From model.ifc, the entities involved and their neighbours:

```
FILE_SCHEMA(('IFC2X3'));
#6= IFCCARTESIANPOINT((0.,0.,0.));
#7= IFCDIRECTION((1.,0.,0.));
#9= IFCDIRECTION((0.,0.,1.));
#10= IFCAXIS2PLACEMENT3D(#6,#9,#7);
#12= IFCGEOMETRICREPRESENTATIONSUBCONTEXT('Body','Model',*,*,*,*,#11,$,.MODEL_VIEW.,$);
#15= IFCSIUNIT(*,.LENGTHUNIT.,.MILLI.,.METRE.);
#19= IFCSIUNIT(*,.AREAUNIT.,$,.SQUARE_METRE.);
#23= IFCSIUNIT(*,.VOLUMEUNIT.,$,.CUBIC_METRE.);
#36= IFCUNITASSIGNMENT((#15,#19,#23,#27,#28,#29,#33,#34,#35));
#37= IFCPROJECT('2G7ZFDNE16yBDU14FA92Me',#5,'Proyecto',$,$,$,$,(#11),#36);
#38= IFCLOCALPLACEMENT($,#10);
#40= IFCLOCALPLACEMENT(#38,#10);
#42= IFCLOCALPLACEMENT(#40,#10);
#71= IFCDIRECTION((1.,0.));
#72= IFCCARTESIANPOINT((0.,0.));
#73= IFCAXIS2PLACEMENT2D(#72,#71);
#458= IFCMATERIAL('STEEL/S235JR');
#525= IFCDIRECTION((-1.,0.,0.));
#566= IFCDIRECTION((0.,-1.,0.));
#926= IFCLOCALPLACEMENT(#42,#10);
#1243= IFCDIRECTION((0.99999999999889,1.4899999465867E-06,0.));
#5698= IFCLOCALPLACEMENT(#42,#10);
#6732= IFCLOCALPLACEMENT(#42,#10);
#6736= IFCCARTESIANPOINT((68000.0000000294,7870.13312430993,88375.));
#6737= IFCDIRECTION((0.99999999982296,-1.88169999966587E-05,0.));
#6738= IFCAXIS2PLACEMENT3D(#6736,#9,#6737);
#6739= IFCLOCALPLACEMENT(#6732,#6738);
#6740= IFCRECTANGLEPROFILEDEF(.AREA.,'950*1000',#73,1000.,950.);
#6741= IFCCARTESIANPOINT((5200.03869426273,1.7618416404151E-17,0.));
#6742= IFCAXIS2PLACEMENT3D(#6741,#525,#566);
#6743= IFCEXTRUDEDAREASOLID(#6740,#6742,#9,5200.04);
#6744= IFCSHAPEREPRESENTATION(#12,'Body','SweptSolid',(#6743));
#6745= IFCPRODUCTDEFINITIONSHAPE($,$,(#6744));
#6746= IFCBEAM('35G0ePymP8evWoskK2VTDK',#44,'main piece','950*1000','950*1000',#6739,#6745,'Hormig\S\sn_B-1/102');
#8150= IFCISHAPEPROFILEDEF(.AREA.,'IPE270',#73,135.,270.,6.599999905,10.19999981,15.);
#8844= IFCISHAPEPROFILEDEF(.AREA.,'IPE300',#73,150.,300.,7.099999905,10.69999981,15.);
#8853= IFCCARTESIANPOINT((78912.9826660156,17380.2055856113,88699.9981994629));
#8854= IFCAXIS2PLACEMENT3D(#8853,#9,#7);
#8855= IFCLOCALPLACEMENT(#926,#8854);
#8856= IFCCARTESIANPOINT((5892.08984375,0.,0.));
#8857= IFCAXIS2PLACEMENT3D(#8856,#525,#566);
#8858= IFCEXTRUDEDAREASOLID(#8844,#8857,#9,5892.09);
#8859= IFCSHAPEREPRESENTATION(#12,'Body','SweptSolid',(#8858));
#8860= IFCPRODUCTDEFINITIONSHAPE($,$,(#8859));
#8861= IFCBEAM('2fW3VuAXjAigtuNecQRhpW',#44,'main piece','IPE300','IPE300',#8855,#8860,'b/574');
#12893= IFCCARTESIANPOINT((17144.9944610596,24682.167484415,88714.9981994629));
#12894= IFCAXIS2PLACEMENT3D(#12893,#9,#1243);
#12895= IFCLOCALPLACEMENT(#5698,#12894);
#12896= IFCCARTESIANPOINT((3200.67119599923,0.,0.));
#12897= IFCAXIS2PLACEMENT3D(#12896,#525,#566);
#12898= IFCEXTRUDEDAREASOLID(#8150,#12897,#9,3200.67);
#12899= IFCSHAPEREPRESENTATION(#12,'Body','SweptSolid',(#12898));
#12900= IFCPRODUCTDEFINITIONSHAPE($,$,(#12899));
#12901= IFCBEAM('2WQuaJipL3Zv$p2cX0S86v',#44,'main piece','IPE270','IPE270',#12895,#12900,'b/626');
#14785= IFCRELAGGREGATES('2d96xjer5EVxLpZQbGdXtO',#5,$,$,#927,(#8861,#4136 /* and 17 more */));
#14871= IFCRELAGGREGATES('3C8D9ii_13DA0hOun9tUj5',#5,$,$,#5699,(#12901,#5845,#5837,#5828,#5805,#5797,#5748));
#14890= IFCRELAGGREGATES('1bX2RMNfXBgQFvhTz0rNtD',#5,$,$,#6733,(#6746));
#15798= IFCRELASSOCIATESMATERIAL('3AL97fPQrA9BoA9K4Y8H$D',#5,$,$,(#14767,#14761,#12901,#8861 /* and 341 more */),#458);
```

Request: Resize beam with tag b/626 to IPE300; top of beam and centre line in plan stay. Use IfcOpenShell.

```python
import ifcopenshell
import ifcopenshell.util.element
import ifcopenshell.util.representation

model = ifcopenshell.open("model.ifc")

member = model.by_id(12901)
source = next(p for p in model.by_type("IfcIShapeProfileDef") if p.ProfileName == "IPE300")

body = ifcopenshell.util.representation.get_representation(member, "Model", "Body")
solid = body.Items[0]
old_profile = solid.SweptArea

# Copy the section's sizes but keep this member's own profile position.
profile = ifcopenshell.util.element.copy(model, source)
# Profiles are centred, so shift by half the change in depth to hold the top.
shift = (old_profile.OverallDepth - profile.OverallDepth) / 2
x, y = old_profile.Position.Location.Coordinates
up = (0.0, 1.0)  # upwards, in the solid's own plane
location = model.createIfcCartesianPoint((x + up[0] * shift, y + up[1] * shift))
profile.Position = model.createIfcAxis2Placement2D(location, old_profile.Position.RefDirection)
solid.SweptArea = profile
if not model.get_total_inverses(old_profile):
    ifcopenshell.util.element.remove_deep2(model, old_profile)
member.Description = member.Description.replace("IPE270", "IPE300")
member.ObjectType = member.ObjectType.replace("IPE270", "IPE300")

print(solid.SweptArea)

model.write("model_updated.ifc")
```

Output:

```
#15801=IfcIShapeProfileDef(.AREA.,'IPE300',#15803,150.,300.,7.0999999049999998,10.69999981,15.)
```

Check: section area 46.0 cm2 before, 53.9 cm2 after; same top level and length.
